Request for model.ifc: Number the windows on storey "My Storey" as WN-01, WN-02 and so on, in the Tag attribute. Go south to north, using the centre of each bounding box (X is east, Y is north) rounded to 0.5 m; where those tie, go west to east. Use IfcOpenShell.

First a look at what the model holds.

```python
import ifcopenshell
import ifcopenshell.util.element
import ifcopenshell.util.placement

model = ifcopenshell.open("model.ifc")
print(model.schema)
storey = next(s for s in model.by_type("IfcBuildingStorey") if s.Name == "My Storey")
windows = [e for e in ifcopenshell.util.element.get_decomposition(storey) if e.is_a("IfcWindow")]
for e in sorted(windows, key=lambda e: e.id()):
    origin = ifcopenshell.util.placement.get_local_placement(e.ObjectPlacement)[:3, 3]
    print(e.id(), e.Tag, e.Name, origin.round(2) + 0.0, sep=" | ")
```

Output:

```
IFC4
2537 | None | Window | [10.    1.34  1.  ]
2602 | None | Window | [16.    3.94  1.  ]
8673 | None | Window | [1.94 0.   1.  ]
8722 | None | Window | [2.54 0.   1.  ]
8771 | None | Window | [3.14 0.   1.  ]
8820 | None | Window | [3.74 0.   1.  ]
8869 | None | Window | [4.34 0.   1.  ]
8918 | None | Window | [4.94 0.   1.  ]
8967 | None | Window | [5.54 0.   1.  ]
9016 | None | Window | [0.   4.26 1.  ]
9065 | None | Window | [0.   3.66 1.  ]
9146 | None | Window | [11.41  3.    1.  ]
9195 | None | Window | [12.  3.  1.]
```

```python
import ifcopenshell
import ifcopenshell.geom
import ifcopenshell.util.element
import ifcopenshell.util.shape

model = ifcopenshell.open("model.ifc")
settings = ifcopenshell.geom.settings()
settings.set("use-world-coords", True)


def centre(element):
    shape = ifcopenshell.geom.create_shape(settings, element)
    return ifcopenshell.util.shape.get_bbox_centroid(shape.geometry)


storey = next(s for s in model.by_type("IfcBuildingStorey") if s.Name == "My Storey")
windows = [e for e in ifcopenshell.util.element.get_decomposition(storey) if e.is_a("IfcWindow")]

# Insertion points can sit at a corner or the storey origin, so sort by the geometry (in metres).
centres = {e: centre(e) for e in windows}
windows.sort(key=lambda e: (round(centres[e][1] / 0.5), centres[e][0]))

for i, e in enumerate(windows, start=1):
    number = f"WN-{i:02d}"
    e.Tag = number
    print(e.id(), number)

model.write("model_v2.ifc")
```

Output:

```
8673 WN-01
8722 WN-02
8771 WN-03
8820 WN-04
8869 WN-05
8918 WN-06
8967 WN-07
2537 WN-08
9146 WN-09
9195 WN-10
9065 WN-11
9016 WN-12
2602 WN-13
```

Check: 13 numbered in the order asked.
